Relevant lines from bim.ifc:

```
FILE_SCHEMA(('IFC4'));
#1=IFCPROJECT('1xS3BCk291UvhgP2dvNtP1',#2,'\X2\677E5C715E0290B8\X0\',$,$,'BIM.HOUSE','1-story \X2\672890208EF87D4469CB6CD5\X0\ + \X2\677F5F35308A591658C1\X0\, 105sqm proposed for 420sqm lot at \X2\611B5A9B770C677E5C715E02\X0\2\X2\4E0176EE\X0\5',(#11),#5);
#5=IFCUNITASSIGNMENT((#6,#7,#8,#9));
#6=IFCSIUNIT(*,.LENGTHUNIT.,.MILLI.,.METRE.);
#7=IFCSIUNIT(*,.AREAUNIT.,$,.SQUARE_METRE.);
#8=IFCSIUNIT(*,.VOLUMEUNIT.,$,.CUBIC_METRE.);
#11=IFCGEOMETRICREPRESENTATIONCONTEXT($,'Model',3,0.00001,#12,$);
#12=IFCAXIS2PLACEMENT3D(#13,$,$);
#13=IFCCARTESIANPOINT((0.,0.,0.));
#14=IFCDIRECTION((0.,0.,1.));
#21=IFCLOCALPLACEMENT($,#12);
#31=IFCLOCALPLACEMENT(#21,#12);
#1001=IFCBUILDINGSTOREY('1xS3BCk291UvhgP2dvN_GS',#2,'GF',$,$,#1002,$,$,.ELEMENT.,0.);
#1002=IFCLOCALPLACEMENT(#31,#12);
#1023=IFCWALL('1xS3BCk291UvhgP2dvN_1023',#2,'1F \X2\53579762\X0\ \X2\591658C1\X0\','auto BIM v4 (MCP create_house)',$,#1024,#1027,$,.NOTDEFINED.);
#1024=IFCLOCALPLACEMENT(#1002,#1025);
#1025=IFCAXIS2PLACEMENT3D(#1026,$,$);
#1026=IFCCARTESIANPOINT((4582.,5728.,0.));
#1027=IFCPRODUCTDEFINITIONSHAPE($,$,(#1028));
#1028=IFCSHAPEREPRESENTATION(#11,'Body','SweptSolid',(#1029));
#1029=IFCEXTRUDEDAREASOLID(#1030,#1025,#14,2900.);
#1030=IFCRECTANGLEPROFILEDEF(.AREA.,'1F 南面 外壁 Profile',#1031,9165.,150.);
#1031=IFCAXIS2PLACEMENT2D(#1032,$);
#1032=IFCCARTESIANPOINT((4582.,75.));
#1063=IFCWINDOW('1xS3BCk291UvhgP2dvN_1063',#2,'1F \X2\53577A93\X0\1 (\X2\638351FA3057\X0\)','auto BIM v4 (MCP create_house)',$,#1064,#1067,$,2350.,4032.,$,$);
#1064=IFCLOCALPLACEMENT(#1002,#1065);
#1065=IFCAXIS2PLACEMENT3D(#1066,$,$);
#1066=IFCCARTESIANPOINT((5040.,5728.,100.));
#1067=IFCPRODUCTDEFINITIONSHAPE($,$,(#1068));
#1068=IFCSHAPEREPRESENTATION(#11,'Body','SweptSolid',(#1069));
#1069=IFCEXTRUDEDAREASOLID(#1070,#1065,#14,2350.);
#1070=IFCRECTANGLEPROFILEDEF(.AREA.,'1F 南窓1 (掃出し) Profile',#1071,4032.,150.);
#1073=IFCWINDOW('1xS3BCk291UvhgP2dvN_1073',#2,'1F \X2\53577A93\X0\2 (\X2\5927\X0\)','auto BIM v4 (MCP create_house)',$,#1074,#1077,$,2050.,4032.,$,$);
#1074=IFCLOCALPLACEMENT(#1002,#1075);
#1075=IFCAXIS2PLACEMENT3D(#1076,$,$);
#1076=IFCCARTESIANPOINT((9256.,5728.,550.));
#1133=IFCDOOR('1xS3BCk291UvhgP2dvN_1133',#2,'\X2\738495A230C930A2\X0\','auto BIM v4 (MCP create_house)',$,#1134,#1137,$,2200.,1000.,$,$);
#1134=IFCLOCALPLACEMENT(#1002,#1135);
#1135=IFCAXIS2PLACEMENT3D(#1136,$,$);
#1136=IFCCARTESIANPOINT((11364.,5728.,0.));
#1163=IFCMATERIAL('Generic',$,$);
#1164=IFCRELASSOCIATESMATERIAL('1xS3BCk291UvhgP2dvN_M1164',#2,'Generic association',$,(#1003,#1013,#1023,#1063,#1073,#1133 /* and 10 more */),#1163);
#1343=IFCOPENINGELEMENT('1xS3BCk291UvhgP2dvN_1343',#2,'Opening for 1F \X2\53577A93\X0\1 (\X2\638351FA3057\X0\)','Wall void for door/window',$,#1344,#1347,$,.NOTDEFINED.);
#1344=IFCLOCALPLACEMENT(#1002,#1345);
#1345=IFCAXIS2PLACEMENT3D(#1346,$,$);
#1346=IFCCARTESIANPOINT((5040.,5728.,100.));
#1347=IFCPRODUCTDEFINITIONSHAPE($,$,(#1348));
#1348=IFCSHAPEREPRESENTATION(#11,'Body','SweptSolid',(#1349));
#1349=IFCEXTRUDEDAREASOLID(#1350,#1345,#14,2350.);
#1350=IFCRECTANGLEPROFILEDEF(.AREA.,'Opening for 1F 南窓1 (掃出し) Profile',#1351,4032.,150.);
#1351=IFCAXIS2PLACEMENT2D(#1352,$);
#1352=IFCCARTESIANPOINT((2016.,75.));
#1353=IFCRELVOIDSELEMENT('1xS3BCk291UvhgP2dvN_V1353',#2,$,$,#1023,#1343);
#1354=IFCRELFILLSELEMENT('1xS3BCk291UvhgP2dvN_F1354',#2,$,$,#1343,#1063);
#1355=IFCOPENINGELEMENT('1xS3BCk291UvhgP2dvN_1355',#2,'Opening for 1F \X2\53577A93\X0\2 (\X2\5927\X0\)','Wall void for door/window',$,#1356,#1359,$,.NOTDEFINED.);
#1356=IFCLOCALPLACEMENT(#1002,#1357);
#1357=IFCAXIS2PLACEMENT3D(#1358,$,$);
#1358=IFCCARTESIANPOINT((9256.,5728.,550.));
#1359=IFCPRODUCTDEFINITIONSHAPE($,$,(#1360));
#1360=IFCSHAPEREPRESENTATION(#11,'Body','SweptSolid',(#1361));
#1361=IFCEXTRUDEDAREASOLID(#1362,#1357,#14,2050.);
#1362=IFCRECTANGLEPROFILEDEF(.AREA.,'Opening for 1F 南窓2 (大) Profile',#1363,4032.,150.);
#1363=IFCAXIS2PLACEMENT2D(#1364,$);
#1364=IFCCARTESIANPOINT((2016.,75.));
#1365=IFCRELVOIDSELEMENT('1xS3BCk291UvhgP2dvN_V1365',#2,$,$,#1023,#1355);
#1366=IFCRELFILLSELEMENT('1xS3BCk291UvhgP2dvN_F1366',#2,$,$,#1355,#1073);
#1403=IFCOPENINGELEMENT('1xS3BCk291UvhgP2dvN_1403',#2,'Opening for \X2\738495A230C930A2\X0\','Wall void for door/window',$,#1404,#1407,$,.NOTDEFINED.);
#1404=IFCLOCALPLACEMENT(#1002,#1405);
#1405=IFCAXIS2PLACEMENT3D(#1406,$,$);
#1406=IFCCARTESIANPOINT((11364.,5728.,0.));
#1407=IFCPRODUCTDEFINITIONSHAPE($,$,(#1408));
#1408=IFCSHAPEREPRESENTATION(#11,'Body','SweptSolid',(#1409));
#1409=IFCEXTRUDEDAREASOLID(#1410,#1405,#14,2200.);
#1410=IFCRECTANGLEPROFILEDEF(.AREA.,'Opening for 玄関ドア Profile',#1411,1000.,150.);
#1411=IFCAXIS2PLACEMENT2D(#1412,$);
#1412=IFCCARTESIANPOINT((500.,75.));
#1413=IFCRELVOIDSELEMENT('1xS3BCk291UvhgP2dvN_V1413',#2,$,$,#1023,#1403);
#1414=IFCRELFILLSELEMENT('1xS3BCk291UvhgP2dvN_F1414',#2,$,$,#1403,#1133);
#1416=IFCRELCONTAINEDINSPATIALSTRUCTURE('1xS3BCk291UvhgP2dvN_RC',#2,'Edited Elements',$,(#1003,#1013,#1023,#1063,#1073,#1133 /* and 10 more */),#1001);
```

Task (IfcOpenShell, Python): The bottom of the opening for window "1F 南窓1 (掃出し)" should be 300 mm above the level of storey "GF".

```python
import numpy as np
import ifcopenshell
import ifcopenshell.api.geometry
import ifcopenshell.geom
import ifcopenshell.util.element
import ifcopenshell.util.placement
import ifcopenshell.util.shape
import ifcopenshell.util.unit

model = ifcopenshell.open("bim.ifc")
unit_scale = ifcopenshell.util.unit.calculate_unit_scale(model)

window = model.by_guid("1xS3BCk291UvhgP2dvN_1063")
opening = window.FillsVoids[0].RelatingOpeningElement
storey = ifcopenshell.util.element.get_container(window, ifc_class="IfcBuildingStorey")
level = ifcopenshell.util.placement.get_local_placement(storey.ObjectPlacement)[2, 3]

# The opening's origin need not be at the sill, so measure its lowest point.
shape = ifcopenshell.geom.create_shape(ifcopenshell.geom.settings(), opening)
bottom = ifcopenshell.util.shape.get_shape_bottom_elevation(shape, shape.geometry) / unit_scale
dz = level + 0.3 / unit_scale - bottom

shift = np.array([0.0, 0.0, dz])
# The window is not placed relative to its opening, so move both.
for product in (opening, window):
    matrix = ifcopenshell.util.placement.get_local_placement(product.ObjectPlacement)
    matrix[:3, 3] += shift
    ifcopenshell.api.geometry.edit_object_placement(model, product=product, matrix=matrix, is_si=False)

print(f"moved by {dz * unit_scale:+.3f} m")

model.write("bim_rev.ifc")
```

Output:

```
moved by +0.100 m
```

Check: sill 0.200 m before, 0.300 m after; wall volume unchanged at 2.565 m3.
